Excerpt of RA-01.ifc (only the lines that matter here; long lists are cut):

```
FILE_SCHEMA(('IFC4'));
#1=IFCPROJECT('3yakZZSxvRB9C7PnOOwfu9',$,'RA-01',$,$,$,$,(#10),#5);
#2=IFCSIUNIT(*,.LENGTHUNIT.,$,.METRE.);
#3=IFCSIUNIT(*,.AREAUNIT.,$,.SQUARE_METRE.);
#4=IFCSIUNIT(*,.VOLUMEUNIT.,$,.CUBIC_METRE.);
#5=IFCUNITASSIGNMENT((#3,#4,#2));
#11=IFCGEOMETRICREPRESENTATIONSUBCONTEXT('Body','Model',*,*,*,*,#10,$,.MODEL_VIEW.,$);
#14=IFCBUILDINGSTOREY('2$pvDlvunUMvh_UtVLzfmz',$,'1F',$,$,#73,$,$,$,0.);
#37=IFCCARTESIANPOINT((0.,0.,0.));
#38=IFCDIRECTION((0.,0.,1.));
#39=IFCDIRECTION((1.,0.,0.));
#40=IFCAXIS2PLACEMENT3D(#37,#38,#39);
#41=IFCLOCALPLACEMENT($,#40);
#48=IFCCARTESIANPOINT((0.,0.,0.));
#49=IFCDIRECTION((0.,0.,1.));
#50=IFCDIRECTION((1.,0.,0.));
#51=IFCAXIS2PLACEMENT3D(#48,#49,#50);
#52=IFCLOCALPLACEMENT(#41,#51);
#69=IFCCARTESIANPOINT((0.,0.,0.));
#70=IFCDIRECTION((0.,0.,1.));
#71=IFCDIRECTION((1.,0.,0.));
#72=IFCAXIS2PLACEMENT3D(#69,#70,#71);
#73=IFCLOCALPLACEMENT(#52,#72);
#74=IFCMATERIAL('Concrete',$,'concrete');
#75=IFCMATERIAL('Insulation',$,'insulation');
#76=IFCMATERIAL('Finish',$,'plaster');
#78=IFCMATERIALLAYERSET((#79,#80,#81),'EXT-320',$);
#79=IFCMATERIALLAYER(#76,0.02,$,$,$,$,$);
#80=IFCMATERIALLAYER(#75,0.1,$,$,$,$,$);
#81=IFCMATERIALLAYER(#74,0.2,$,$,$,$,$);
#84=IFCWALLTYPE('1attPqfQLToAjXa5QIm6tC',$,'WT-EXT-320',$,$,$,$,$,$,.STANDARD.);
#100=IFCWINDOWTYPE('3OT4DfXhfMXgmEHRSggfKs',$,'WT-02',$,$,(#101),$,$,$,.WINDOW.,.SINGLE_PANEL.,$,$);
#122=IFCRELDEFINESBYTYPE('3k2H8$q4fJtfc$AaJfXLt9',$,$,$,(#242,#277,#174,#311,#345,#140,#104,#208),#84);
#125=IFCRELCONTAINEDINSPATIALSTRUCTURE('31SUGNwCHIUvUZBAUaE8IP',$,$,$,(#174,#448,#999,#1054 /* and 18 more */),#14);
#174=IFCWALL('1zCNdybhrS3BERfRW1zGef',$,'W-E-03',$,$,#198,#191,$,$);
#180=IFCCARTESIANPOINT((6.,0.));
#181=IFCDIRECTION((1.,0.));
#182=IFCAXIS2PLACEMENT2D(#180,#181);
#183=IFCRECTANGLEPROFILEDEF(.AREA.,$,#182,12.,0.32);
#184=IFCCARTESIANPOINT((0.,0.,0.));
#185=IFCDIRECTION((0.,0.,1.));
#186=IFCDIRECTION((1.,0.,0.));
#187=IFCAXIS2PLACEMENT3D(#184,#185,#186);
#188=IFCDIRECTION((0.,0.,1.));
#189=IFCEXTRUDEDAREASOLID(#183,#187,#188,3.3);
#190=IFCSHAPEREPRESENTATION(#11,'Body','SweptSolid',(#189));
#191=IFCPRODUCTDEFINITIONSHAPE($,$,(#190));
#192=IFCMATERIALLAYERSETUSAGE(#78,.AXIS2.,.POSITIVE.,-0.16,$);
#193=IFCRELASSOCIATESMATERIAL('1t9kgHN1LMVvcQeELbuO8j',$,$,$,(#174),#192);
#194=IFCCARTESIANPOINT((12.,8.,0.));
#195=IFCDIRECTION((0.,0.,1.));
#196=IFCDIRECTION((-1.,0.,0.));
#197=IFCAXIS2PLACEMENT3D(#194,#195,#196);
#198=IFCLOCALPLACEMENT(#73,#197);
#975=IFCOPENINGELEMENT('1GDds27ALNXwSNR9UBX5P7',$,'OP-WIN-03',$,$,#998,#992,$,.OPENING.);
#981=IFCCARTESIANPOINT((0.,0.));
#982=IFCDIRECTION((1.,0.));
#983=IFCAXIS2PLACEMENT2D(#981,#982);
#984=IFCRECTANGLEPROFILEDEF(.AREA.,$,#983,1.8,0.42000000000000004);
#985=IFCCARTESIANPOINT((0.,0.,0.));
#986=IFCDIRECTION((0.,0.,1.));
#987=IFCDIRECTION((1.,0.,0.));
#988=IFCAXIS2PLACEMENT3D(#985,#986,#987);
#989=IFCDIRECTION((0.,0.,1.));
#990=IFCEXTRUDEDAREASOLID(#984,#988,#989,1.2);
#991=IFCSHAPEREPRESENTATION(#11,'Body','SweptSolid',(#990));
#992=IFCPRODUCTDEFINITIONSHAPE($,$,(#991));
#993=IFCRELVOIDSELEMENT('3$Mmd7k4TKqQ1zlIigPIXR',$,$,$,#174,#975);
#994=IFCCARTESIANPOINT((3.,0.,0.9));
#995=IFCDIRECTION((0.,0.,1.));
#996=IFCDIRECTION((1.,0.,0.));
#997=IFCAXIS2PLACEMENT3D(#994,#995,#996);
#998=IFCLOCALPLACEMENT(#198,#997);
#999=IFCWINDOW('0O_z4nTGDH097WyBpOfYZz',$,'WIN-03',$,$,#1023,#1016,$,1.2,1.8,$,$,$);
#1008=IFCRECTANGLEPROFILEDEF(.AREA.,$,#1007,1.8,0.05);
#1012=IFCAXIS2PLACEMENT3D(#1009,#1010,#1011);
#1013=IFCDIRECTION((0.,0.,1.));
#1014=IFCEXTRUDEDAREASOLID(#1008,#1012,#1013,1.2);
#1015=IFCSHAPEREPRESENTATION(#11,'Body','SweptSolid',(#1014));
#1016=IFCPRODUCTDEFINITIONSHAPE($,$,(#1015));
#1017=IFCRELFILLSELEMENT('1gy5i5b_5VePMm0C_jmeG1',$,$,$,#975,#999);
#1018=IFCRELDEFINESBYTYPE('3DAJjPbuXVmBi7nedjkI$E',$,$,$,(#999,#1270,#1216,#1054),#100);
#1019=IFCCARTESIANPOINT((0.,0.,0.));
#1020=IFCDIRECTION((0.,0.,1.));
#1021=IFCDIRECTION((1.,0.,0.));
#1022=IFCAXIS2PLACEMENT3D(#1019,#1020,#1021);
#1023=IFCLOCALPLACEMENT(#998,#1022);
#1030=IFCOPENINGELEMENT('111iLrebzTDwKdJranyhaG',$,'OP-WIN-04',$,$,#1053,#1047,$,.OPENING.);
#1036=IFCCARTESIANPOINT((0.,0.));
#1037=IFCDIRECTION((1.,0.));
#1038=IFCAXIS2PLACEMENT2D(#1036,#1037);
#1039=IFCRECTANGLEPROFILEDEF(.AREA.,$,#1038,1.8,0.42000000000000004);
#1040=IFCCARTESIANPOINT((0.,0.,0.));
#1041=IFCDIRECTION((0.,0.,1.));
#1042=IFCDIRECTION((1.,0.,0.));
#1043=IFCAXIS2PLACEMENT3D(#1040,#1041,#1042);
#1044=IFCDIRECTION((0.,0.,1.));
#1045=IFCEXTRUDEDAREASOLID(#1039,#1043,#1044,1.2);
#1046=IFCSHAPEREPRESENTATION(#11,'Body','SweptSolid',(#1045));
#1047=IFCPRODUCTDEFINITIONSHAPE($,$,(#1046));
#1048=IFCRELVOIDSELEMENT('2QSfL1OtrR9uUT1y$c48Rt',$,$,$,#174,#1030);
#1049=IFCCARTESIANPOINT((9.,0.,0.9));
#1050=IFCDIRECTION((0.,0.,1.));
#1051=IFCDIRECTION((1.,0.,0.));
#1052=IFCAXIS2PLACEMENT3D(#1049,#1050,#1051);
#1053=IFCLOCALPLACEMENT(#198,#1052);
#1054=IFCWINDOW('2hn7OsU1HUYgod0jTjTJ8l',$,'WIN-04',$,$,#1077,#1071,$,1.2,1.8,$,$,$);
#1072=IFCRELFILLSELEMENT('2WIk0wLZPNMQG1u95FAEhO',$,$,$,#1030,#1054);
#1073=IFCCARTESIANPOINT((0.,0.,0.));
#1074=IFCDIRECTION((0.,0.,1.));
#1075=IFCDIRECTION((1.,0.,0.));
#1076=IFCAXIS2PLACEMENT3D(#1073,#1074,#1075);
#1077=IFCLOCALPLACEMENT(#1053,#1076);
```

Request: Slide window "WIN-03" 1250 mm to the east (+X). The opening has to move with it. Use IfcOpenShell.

```python
import ifcopenshell
import ifcopenshell.api.geometry
import ifcopenshell.util.placement

model = ifcopenshell.open("RA-01.ifc")

window = model.by_id(999)
opening = window.FillsVoids[0].RelatingOpeningElement
wall = opening.VoidsElements[0].RelatingBuildingElement

wall_matrix = ifcopenshell.util.placement.get_local_placement(wall.ObjectPlacement)
shift = wall_matrix[:3, 0] * -1.25
before = ifcopenshell.util.placement.get_local_placement(window.ObjectPlacement)[:3, 3].copy()

# The window is placed relative to its opening, so it follows when the opening moves.
matrix = ifcopenshell.util.placement.get_local_placement(opening.ObjectPlacement)
matrix[:3, 3] += shift
ifcopenshell.api.geometry.edit_object_placement(
    model, product=opening, matrix=matrix, is_si=False, should_transform_children=True
)

after = ifcopenshell.util.placement.get_local_placement(window.ObjectPlacement)[:3, 3]
print("window moved by", (after - before).round(3) + 0.0)

model.write("RA-01_rev.ifc")
```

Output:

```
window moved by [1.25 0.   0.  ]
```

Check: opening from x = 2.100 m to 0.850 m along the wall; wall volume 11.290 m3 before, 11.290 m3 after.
